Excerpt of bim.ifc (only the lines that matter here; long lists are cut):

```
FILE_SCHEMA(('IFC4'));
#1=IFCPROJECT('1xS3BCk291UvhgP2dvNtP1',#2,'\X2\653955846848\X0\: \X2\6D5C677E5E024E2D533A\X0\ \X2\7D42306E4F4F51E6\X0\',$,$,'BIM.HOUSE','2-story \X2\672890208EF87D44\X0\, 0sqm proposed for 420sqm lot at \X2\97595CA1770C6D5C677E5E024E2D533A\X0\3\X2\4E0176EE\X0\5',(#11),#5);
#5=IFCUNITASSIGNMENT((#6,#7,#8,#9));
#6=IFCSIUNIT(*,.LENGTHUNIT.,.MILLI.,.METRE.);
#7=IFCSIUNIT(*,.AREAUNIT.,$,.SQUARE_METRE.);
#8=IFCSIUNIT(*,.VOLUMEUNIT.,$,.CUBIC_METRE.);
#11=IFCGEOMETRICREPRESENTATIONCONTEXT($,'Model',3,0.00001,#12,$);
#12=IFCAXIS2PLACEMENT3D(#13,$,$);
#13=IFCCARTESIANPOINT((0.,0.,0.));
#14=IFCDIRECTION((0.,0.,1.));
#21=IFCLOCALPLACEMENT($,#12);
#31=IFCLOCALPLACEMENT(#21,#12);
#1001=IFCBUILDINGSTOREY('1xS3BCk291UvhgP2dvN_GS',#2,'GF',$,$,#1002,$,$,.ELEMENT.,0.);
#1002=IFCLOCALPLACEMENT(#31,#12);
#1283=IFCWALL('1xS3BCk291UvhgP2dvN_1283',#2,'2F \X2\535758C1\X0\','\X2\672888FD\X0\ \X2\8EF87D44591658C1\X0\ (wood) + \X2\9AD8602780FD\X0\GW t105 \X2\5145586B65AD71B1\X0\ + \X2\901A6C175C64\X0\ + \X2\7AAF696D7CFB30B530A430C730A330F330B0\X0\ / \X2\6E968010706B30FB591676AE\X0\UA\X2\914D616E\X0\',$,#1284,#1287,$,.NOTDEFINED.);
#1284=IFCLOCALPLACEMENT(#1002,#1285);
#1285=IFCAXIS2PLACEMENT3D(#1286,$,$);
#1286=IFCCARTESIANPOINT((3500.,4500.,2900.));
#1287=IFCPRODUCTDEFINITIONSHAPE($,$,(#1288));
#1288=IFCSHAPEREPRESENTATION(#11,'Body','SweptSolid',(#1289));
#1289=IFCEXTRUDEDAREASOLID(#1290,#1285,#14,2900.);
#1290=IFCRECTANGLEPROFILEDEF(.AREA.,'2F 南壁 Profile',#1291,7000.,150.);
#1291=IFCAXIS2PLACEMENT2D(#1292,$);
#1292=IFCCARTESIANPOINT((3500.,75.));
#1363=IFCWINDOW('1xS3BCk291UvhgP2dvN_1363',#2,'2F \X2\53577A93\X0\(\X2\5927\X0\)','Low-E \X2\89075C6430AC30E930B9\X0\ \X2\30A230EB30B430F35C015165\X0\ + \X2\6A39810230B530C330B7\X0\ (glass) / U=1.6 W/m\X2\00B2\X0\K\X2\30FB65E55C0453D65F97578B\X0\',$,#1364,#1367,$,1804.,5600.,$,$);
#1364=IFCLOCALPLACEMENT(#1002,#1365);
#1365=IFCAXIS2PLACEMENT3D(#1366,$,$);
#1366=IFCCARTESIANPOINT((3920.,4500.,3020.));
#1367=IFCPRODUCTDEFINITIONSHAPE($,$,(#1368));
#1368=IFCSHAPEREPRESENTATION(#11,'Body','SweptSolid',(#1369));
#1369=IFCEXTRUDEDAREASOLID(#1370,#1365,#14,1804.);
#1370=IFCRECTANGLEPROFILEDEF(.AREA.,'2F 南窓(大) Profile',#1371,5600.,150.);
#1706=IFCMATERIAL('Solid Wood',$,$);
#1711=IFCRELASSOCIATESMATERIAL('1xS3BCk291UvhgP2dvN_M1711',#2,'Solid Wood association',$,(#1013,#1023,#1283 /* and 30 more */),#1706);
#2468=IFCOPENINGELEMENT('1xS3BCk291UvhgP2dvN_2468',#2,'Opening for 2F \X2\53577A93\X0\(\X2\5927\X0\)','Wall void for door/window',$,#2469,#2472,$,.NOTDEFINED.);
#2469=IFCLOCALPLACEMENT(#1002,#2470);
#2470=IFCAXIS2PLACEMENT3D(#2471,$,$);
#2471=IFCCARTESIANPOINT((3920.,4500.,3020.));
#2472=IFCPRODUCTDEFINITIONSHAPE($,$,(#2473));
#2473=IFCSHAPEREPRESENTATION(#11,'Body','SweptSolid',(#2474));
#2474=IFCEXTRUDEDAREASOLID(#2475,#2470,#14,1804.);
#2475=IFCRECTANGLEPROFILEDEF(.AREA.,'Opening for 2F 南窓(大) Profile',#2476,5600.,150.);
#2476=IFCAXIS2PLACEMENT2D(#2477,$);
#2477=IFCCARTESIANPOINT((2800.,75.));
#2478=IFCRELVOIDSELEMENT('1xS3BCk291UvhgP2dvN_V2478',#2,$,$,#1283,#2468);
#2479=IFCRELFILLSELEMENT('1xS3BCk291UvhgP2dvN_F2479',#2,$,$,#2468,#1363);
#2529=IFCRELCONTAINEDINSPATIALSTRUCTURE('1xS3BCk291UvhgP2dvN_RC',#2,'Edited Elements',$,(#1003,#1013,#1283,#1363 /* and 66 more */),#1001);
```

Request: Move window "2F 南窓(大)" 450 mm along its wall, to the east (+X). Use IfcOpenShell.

```python
import ifcopenshell
import ifcopenshell.api.geometry
import ifcopenshell.util.placement
import ifcopenshell.util.unit

model = ifcopenshell.open("bim.ifc")
unit_scale = ifcopenshell.util.unit.calculate_unit_scale(model)

window = model.by_id(1363)
opening = window.FillsVoids[0].RelatingOpeningElement
wall = opening.VoidsElements[0].RelatingBuildingElement

wall_matrix = ifcopenshell.util.placement.get_local_placement(wall.ObjectPlacement)
shift = wall_matrix[:3, 0] * 0.45 / unit_scale
before = ifcopenshell.util.placement.get_local_placement(window.ObjectPlacement)[:3, 3].copy()

# The window is not placed relative to its opening, so move both.
for product in (opening, window):
    matrix = ifcopenshell.util.placement.get_local_placement(product.ObjectPlacement)
    matrix[:3, 3] += shift
    ifcopenshell.api.geometry.edit_object_placement(model, product=product, matrix=matrix, is_si=False)

after = ifcopenshell.util.placement.get_local_placement(window.ObjectPlacement)[:3, 3]
print("window moved by", (after - before).round(3) + 0.0)

model.write("bim-out.ifc")
```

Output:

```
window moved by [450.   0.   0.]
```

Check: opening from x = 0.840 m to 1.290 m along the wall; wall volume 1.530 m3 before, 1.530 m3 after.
